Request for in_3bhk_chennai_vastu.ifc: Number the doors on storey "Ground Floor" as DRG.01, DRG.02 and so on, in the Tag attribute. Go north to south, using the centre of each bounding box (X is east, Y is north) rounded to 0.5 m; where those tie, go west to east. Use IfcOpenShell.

First a look at what the model holds.

```python
import ifcopenshell
import ifcopenshell.util.element
import ifcopenshell.util.placement

model = ifcopenshell.open("in_3bhk_chennai_vastu.ifc")
print(model.schema)
storey = next(s for s in model.by_type("IfcBuildingStorey") if s.Name == "Ground Floor")
doors = [e for e in ifcopenshell.util.element.get_decomposition(storey) if e.is_a("IfcDoor")]
for e in sorted(doors, key=lambda e: e.id()):
    origin = ifcopenshell.util.placement.get_local_placement(e.ObjectPlacement)[:3, 3]
    print(e.id(), e.Tag, e.Name, origin.round(2) + 0.0, sep=" | ")
```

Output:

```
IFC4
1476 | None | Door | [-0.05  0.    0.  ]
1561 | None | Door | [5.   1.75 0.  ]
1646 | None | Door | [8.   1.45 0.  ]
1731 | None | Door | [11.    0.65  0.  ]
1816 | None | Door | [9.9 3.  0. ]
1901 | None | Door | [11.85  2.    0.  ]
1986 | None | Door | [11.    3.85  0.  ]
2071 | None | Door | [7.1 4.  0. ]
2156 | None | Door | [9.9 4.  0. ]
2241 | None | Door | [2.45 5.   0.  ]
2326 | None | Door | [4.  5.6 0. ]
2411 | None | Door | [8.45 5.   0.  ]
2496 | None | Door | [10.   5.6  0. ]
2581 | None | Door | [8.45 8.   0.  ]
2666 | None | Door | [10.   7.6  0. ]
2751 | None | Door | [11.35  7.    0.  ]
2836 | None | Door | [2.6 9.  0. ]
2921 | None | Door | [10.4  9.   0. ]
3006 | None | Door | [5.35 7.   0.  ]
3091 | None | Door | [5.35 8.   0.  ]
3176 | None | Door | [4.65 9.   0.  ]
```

```python
import ifcopenshell
import ifcopenshell.geom
import ifcopenshell.util.element
import ifcopenshell.util.shape

model = ifcopenshell.open("in_3bhk_chennai_vastu.ifc")
settings = ifcopenshell.geom.settings()
settings.set("use-world-coords", True)


def centre(element):
    shape = ifcopenshell.geom.create_shape(settings, element)
    return ifcopenshell.util.shape.get_bbox_centroid(shape.geometry)


storey = next(s for s in model.by_type("IfcBuildingStorey") if s.Name == "Ground Floor")
doors = [e for e in ifcopenshell.util.element.get_decomposition(storey) if e.is_a("IfcDoor")]

# Insertion points can sit at a corner or the storey origin, so sort by the geometry (in metres).
centres = {e: centre(e) for e in doors}
doors.sort(key=lambda e: (-round(centres[e][1] / 0.5), centres[e][0]))

for i, e in enumerate(doors, start=1):
    number = f"DRG.{i:02d}"
    e.Tag = number
    print(e.id(), number)

model.write("in_3bhk_chennai_vastu_v2.ifc")
```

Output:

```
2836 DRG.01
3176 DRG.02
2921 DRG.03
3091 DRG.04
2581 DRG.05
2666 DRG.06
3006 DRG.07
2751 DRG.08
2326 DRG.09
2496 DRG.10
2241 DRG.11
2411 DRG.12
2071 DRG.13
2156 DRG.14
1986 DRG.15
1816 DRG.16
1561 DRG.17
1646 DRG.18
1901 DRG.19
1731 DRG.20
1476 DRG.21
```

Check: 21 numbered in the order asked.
